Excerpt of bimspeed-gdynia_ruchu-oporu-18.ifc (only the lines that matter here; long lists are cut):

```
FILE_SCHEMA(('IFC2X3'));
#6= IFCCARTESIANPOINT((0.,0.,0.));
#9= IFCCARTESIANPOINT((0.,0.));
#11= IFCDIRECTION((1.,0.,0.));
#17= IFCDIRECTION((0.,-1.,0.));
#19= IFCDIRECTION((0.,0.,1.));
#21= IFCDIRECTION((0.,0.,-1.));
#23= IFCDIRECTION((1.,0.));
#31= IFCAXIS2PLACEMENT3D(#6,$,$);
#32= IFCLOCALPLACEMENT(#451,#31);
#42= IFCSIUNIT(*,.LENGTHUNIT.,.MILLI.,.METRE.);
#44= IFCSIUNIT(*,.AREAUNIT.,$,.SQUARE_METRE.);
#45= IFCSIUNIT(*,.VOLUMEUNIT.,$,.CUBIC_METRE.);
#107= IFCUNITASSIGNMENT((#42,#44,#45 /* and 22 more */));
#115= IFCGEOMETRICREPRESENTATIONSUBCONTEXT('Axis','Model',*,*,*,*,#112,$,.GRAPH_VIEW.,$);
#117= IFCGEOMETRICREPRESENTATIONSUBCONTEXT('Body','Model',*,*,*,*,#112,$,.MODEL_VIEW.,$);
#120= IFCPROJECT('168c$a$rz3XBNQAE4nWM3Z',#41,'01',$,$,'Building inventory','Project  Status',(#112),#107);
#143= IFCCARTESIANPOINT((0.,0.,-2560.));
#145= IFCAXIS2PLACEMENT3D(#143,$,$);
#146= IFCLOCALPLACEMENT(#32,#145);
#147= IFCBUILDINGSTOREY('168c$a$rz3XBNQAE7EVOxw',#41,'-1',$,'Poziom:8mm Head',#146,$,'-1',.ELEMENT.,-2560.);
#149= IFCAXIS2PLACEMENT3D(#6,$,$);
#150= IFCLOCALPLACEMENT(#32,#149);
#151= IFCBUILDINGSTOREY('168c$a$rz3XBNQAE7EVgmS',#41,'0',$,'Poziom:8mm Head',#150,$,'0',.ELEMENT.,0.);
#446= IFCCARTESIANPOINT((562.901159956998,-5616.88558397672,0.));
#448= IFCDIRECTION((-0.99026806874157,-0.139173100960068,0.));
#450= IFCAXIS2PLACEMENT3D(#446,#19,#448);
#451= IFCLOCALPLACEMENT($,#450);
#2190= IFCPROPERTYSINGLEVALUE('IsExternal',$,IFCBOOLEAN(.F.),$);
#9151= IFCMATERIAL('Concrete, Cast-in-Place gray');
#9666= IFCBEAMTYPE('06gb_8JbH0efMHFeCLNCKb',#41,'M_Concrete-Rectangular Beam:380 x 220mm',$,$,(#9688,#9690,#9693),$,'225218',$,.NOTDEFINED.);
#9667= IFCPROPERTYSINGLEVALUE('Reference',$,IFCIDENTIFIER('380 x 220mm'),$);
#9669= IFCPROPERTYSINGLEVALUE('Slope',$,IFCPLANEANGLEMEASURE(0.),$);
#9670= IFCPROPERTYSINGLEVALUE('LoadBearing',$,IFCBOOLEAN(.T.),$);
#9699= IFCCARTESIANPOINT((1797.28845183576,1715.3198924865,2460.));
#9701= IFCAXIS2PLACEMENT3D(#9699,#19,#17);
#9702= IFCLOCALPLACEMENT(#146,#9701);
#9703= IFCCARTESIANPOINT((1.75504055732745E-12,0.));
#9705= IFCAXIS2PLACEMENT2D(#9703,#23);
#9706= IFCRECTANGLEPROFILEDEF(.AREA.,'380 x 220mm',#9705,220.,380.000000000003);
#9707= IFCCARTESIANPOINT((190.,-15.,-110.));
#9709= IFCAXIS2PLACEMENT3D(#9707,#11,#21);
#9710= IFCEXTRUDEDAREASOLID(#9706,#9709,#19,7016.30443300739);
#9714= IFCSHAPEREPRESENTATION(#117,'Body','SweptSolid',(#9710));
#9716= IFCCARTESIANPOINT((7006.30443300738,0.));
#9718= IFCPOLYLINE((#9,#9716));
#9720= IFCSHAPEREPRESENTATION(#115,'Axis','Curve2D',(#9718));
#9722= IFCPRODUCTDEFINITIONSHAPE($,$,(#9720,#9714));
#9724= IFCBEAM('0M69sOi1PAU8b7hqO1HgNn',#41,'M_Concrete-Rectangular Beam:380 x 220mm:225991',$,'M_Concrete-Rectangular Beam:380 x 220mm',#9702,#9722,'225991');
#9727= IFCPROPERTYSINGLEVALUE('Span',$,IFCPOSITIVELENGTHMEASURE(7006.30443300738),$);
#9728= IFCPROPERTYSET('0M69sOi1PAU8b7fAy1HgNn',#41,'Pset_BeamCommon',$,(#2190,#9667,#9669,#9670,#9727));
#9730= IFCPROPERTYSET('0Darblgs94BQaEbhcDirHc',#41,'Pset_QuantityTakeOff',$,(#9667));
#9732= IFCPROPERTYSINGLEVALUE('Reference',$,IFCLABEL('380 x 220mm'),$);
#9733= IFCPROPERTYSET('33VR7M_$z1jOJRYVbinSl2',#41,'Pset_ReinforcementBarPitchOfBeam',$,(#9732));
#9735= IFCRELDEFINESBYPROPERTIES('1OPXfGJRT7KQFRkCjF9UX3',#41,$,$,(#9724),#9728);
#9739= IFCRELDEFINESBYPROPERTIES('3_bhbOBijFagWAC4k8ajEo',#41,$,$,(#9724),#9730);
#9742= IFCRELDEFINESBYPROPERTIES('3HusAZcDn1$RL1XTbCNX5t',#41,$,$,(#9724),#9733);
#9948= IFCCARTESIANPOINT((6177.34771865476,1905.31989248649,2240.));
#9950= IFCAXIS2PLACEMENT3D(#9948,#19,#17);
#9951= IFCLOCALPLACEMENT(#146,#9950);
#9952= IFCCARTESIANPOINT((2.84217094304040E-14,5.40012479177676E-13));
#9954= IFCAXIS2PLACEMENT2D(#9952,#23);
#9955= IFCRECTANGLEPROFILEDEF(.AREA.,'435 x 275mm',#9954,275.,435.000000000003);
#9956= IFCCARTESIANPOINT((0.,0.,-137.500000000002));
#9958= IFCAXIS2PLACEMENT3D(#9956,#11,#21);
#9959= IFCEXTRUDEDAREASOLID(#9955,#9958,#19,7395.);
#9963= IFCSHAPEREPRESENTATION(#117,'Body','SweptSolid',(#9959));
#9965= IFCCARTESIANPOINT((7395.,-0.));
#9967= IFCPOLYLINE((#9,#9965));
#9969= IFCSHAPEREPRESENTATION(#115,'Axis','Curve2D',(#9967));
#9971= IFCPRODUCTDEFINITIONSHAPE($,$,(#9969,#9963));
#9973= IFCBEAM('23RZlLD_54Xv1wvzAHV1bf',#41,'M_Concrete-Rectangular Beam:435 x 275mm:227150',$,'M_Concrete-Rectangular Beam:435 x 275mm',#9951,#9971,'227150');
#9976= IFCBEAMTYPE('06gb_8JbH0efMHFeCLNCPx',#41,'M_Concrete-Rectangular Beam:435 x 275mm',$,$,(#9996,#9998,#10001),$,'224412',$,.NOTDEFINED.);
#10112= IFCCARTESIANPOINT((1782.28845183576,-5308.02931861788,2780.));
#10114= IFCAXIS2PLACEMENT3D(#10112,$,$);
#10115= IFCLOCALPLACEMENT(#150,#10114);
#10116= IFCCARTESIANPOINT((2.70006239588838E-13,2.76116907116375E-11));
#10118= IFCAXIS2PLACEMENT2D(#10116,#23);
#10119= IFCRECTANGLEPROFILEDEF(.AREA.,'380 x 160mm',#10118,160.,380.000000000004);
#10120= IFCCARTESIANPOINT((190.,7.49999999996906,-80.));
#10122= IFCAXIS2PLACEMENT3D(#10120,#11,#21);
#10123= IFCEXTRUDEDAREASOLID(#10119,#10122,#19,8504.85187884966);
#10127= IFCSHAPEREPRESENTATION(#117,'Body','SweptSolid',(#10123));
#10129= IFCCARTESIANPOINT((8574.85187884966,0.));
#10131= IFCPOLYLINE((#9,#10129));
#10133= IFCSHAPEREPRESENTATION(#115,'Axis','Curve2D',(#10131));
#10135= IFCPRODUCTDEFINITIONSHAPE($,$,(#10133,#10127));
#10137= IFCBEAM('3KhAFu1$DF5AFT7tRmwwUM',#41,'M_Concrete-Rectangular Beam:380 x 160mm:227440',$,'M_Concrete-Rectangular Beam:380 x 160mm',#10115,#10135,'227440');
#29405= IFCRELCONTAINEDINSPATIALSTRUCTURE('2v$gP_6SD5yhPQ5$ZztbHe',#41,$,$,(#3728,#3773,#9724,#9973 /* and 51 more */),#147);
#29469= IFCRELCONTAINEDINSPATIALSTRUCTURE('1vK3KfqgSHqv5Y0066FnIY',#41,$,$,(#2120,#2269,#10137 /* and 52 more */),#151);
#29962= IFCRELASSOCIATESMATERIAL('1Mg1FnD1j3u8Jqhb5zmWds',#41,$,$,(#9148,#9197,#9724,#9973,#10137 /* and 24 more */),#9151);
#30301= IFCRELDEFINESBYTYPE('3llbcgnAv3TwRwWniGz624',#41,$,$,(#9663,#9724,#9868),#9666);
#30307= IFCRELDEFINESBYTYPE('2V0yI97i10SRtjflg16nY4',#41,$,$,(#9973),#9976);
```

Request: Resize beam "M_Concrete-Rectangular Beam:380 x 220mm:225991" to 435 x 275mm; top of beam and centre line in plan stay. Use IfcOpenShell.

```python
import ifcopenshell
import ifcopenshell.api.pset
import ifcopenshell.api.type
import ifcopenshell.util.element
import ifcopenshell.util.representation

model = ifcopenshell.open("bimspeed-gdynia_ruchu-oporu-18.ifc")

member = model.by_guid("0M69sOi1PAU8b7hqO1HgNn")
source = next(p for p in model.by_type("IfcRectangleProfileDef") if p.ProfileName == "435 x 275mm")

body = ifcopenshell.util.representation.get_representation(member, "Model", "Body")
solid = body.Items[0]
old_profile = solid.SweptArea

# Copy the section's sizes but keep this member's own profile position.
profile = ifcopenshell.util.element.copy(model, source)
# Profiles are centred, so shift by half the change in depth to hold the top.
shift = (old_profile.XDim - profile.XDim) / 2
x, y = old_profile.Position.Location.Coordinates
up = (-1.0, 0.0)  # upwards, in the solid's own plane
location = model.createIfcCartesianPoint((x + up[0] * shift, y + up[1] * shift))
profile.Position = model.createIfcAxis2Placement2D(location, old_profile.Position.RefDirection)
solid.SweptArea = profile
if not model.get_total_inverses(old_profile):
    ifcopenshell.util.element.remove_deep2(model, old_profile)

new_type = model.by_guid("06gb_8JbH0efMHFeCLNCPx")
ifcopenshell.api.type.assign_type(
    model, related_objects=[member], relating_type=new_type, should_map_representations=False
)
member.Name = member.Name.replace("380 x 220mm", "435 x 275mm")
member.ObjectType = "M_Concrete-Rectangular Beam:435 x 275mm"
pset = model.by_id(ifcopenshell.util.element.get_pset(member, "Pset_BeamCommon", should_inherit=False)["id"])
ifcopenshell.api.pset.edit_pset(model, pset=pset, properties={"Reference": "435 x 275mm"})
pset = model.by_id(ifcopenshell.util.element.get_pset(member, "Pset_QuantityTakeOff", should_inherit=False)["id"])
ifcopenshell.api.pset.edit_pset(model, pset=pset, properties={"Reference": "435 x 275mm"})
pset = model.by_id(ifcopenshell.util.element.get_pset(member, "Pset_ReinforcementBarPitchOfBeam", should_inherit=False)["id"])
ifcopenshell.api.pset.edit_pset(model, pset=pset, properties={"Reference": "435 x 275mm"})

print(solid.SweptArea)

model.write("bimspeed-gdynia_ruchu-oporu-18_updated.ifc")
```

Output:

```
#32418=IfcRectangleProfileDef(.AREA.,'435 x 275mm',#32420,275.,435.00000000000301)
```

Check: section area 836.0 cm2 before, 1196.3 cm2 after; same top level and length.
